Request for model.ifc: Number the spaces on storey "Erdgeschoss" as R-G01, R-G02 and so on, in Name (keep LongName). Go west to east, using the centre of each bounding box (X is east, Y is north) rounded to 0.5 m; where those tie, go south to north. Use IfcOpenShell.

First a look at what the model holds.

```python
import ifcopenshell
import ifcopenshell.util.element
import ifcopenshell.util.placement

model = ifcopenshell.open("model.ifc")
print(model.schema)
storey = next(s for s in model.by_type("IfcBuildingStorey") if s.Name == "Erdgeschoss")
spaces = [e for e in ifcopenshell.util.element.get_decomposition(storey) if e.is_a("IfcSpace")]
for e in sorted(spaces, key=lambda e: e.id()):
    origin = ifcopenshell.util.placement.get_local_placement(e.ObjectPlacement)[:3, 3]
    print(e.id(), e.Name, e.LongName, origin.round(2) + 0.0, sep=" | ")
```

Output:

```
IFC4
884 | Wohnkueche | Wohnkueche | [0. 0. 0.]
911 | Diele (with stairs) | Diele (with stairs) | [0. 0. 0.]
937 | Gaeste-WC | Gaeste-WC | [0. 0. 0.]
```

```python
import ifcopenshell
import ifcopenshell.geom
import ifcopenshell.util.element
import ifcopenshell.util.shape

model = ifcopenshell.open("model.ifc")
settings = ifcopenshell.geom.settings()
settings.set("use-world-coords", True)


def centre(element):
    shape = ifcopenshell.geom.create_shape(settings, element)
    return ifcopenshell.util.shape.get_bbox_centroid(shape.geometry)


storey = next(s for s in model.by_type("IfcBuildingStorey") if s.Name == "Erdgeschoss")
spaces = [e for e in ifcopenshell.util.element.get_decomposition(storey) if e.is_a("IfcSpace")]

# Insertion points can sit at a corner or the storey origin, so sort by the geometry (in metres).
centres = {e: centre(e) for e in spaces}
spaces.sort(key=lambda e: (round(centres[e][0] / 0.5), centres[e][1]))

for i, e in enumerate(spaces, start=1):
    number = f"R-G{i:02d}"
    e.Name = number
    print(e.id(), number)

model.write("model_v2.ifc")
```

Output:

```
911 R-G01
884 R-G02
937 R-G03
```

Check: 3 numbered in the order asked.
